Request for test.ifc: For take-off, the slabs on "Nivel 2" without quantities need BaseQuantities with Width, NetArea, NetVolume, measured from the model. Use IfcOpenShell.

First a look at what the model holds.

```python
import ifcopenshell
import ifcopenshell.util.element
import ifcopenshell.util.unit

model = ifcopenshell.open("test.ifc")
print(model.schema)
for unit_type in ("LENGTHUNIT", "AREAUNIT", "VOLUMEUNIT"):
    print(unit_type, ifcopenshell.util.unit.calculate_unit_scale(model, unit_type))
storey = next(s for s in model.by_type("IfcBuildingStorey") if s.Name == "Nivel 2")
slabs = [e for e in ifcopenshell.util.element.get_decomposition(storey) if e.is_a("IfcSlab")]
for e in sorted(slabs, key=lambda e: e.id()):
    print(e.id(), e.is_a(), e.Name, list(ifcopenshell.util.element.get_psets(e, qtos_only=True)), sep=" | ")
```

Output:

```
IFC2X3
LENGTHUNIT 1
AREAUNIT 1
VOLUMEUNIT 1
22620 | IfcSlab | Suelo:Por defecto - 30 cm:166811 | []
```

```python
import ifcopenshell
import ifcopenshell.api.pset
import ifcopenshell.geom
import ifcopenshell.util.element
import ifcopenshell.util.shape
import ifcopenshell.util.unit

model = ifcopenshell.open("test.ifc")
unit_scale = ifcopenshell.util.unit.calculate_unit_scale(model)
area_scale = ifcopenshell.util.unit.calculate_unit_scale(model, "AREAUNIT")
volume_scale = ifcopenshell.util.unit.calculate_unit_scale(model, "VOLUMEUNIT")
settings = ifcopenshell.geom.settings()

storey = next(s for s in model.by_type("IfcBuildingStorey") if s.Name == "Nivel 2")
slabs = [e for e in ifcopenshell.util.element.get_decomposition(storey) if e.is_a("IfcSlab")]

for e in sorted(slabs, key=lambda e: e.id()):
    if ifcopenshell.util.element.get_psets(e, qtos_only=True, should_inherit=False):
        continue
    # Geometry comes back in metres, in the element's own axes.
    shape = ifcopenshell.geom.create_shape(settings, e)
    values = {
        "Width": ifcopenshell.util.shape.get_z(shape.geometry) / unit_scale,
        "NetArea": ifcopenshell.util.shape.get_footprint_area(shape.geometry) / area_scale,
        "NetVolume": ifcopenshell.util.shape.get_volume(shape.geometry) / volume_scale,
    }
    qto = ifcopenshell.api.pset.add_qto(model, product=e, name="BaseQuantities")
    ifcopenshell.api.pset.edit_qto(model, qto=qto, properties=values)
    print(e.id(), {k: round(v, 3) for k, v in values.items()})

model.write("test_rev.ifc")
```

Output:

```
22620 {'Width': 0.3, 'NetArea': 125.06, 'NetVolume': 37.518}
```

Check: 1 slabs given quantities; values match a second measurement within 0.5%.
